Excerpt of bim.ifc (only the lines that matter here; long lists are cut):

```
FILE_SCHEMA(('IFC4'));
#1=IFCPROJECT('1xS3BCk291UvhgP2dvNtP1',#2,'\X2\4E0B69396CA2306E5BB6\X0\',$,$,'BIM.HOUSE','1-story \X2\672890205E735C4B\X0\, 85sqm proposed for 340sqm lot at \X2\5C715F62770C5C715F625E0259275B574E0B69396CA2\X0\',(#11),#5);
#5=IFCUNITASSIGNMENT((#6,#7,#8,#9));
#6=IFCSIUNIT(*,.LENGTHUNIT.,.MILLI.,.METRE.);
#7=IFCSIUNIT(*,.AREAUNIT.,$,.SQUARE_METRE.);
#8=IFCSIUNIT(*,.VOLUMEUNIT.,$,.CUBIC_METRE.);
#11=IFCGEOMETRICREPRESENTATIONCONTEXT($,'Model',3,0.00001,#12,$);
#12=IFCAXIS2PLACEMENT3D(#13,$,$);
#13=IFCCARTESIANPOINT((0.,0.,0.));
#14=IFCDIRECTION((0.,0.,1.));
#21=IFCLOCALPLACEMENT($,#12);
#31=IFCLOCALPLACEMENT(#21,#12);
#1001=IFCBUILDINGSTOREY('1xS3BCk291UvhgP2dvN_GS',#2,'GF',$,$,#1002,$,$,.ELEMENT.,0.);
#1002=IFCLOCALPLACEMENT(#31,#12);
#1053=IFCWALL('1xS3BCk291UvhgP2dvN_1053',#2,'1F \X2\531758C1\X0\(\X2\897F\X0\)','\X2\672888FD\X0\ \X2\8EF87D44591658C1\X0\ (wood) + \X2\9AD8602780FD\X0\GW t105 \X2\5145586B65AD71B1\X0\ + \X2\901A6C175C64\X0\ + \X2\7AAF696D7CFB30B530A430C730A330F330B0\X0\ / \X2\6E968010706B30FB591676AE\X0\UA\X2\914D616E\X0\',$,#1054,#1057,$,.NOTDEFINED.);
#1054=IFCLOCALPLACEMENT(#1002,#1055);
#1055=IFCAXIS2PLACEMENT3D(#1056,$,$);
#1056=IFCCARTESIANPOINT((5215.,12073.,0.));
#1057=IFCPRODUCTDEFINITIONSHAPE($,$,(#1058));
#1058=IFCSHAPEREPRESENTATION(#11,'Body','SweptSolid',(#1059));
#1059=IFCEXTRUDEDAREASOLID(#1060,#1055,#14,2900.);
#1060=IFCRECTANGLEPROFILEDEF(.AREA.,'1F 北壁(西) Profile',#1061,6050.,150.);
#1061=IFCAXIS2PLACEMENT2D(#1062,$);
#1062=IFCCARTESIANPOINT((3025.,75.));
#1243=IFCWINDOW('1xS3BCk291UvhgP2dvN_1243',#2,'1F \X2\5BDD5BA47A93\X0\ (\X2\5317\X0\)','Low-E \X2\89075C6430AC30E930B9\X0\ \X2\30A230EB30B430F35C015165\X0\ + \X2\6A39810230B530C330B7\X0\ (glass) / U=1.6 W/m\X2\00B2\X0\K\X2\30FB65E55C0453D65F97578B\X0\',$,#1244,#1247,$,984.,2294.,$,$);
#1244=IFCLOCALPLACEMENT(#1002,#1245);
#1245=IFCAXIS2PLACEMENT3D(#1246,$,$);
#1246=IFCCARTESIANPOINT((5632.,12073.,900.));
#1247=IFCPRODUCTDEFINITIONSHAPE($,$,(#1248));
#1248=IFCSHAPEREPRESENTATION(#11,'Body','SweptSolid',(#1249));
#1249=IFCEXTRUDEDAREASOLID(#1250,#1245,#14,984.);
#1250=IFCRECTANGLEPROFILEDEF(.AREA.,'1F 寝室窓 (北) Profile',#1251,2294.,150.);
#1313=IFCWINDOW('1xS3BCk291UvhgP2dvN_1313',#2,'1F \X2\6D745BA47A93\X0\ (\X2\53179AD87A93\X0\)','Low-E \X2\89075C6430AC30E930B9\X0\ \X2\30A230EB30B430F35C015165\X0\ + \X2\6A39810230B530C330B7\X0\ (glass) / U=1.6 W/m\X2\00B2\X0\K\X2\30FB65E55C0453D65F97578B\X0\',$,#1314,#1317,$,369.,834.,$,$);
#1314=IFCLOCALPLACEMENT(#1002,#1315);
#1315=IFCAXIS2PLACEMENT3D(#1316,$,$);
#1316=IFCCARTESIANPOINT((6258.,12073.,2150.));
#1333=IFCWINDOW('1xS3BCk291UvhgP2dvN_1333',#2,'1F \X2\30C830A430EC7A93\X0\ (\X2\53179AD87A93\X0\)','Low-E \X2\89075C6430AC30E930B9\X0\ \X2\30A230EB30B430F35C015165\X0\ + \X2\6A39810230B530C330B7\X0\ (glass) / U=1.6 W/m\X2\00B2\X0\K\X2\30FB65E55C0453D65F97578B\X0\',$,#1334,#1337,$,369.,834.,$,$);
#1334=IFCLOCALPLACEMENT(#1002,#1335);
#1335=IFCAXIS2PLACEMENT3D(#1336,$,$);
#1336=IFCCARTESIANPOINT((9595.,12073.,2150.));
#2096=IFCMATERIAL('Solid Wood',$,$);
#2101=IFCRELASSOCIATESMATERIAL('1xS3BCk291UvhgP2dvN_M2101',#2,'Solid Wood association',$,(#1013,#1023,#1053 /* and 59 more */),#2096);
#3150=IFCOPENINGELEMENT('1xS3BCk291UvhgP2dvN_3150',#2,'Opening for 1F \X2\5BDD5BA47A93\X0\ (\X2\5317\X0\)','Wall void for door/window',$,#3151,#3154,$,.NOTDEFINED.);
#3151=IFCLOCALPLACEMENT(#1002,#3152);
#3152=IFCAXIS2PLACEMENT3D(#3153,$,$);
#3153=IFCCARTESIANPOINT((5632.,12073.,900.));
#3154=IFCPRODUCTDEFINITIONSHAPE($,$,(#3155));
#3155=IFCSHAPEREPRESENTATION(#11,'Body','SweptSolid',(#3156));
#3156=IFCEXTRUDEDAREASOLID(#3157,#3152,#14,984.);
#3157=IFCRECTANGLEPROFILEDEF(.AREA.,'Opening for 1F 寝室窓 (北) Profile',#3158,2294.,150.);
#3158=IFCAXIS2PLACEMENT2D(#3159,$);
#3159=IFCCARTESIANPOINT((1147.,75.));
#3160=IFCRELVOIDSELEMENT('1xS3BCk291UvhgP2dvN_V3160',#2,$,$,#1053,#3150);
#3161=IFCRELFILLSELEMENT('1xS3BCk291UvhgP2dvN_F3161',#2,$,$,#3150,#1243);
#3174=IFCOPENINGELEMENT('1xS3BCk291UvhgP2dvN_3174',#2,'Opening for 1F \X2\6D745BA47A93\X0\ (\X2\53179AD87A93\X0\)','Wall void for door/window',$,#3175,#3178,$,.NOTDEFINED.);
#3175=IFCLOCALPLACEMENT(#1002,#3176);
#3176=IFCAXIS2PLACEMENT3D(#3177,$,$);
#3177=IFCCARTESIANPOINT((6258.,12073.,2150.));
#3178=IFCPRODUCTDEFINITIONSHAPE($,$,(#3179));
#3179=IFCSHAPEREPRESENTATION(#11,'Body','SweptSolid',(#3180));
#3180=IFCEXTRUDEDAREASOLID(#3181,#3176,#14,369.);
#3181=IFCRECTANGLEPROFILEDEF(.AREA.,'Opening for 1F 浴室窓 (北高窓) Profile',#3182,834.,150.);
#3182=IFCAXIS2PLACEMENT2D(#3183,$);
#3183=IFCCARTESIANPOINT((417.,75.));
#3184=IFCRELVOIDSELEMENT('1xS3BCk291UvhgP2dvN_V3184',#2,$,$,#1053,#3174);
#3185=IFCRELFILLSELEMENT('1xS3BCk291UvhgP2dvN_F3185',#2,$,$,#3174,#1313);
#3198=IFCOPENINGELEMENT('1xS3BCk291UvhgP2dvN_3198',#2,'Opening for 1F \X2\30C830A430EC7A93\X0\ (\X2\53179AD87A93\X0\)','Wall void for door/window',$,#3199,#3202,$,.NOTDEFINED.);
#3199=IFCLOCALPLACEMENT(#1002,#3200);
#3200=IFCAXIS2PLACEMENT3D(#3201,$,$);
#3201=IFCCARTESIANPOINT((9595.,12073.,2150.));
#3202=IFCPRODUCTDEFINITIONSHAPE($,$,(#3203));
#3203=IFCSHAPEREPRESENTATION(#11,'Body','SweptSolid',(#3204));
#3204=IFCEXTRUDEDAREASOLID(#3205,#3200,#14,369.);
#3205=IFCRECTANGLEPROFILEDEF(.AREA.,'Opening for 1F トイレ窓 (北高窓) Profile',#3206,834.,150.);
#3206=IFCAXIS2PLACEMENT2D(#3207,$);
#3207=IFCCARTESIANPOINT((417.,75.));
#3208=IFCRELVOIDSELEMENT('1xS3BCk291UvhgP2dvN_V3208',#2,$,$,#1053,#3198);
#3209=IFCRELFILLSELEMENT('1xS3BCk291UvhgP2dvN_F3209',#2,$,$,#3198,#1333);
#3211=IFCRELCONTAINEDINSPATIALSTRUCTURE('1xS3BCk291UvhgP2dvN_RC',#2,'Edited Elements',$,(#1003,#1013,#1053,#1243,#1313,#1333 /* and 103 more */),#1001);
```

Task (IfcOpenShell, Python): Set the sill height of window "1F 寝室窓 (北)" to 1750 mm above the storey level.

```python
import numpy as np
import ifcopenshell
import ifcopenshell.api.geometry
import ifcopenshell.geom
import ifcopenshell.util.element
import ifcopenshell.util.placement
import ifcopenshell.util.shape
import ifcopenshell.util.unit

model = ifcopenshell.open("bim.ifc")
unit_scale = ifcopenshell.util.unit.calculate_unit_scale(model)

window = model.by_guid("1xS3BCk291UvhgP2dvN_1243")
opening = window.FillsVoids[0].RelatingOpeningElement
storey = ifcopenshell.util.element.get_container(window, ifc_class="IfcBuildingStorey")
level = ifcopenshell.util.placement.get_local_placement(storey.ObjectPlacement)[2, 3]

# The opening's origin need not be at the sill, so measure its lowest point.
shape = ifcopenshell.geom.create_shape(ifcopenshell.geom.settings(), opening)
bottom = ifcopenshell.util.shape.get_shape_bottom_elevation(shape, shape.geometry) / unit_scale
dz = level + 1750.0 - bottom

shift = np.array([0.0, 0.0, dz])
# The window is not placed relative to its opening, so move both.
for product in (opening, window):
    matrix = ifcopenshell.util.placement.get_local_placement(product.ObjectPlacement)
    matrix[:3, 3] += shift
    ifcopenshell.api.geometry.edit_object_placement(model, product=product, matrix=matrix, is_si=False)

print(f"moved by {dz * unit_scale:+.3f} m")

model.write("bim-out.ifc")
```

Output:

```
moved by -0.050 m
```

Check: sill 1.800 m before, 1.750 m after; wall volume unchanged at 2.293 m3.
